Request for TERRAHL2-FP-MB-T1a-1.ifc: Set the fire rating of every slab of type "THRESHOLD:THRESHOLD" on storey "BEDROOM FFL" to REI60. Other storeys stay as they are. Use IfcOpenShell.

First a look at what the model holds.

```python
import ifcopenshell
import ifcopenshell.util.element

model = ifcopenshell.open("TERRAHL2-FP-MB-T1a-1.ifc")
print(model.schema)
storey = next(s for s in model.by_type("IfcBuildingStorey") if s.Name == "BEDROOM FFL")
slabs = [e for e in ifcopenshell.util.element.get_decomposition(storey) if e.is_a("IfcSlab")]
seen = {}
for e in slabs:
    element_type = ifcopenshell.util.element.get_type(e)
    key = (element_type.Name if element_type != e and element_type else None, ifcopenshell.util.element.get_pset(e, "Pset_SlabCommon", "FireRating"))
    seen[key] = seen.get(key, 0) + 1
for (name, value), count in sorted(seen.items(), key=str):
    print(count, "x", name, "|", value)
```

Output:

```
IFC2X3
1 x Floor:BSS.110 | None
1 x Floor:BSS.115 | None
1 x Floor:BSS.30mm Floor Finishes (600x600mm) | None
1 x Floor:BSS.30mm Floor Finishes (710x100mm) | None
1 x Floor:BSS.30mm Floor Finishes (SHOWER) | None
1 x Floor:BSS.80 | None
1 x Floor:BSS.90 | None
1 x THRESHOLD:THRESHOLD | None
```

```python
import ifcopenshell
import ifcopenshell.api.pset
import ifcopenshell.util.element

model = ifcopenshell.open("TERRAHL2-FP-MB-T1a-1.ifc")

storey = next(s for s in model.by_type("IfcBuildingStorey") if s.Name == "BEDROOM FFL")
slabs = [e for e in ifcopenshell.util.element.get_decomposition(storey) if e.is_a("IfcSlab")]

count = 0
for e in slabs:
    element_type = ifcopenshell.util.element.get_type(e)
    if element_type in (None, e) or element_type.Name != "THRESHOLD:THRESHOLD":
        continue
    # add_pset returns the element's existing set when there is one.
    pset = ifcopenshell.api.pset.add_pset(model, product=e, name="Pset_SlabCommon")
    ifcopenshell.api.pset.edit_pset(model, pset=pset, properties={"FireRating": "REI60"})
    count += 1

print(count, "slabs updated")

model.write("TERRAHL2-FP-MB-T1a-1_v2.ifc")
```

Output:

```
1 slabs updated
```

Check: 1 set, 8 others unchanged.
